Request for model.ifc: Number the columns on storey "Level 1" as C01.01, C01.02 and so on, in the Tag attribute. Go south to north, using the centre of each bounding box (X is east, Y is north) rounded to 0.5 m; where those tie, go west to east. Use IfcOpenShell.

First a look at what the model holds.

```python
import ifcopenshell
import ifcopenshell.util.element
import ifcopenshell.util.placement

model = ifcopenshell.open("model.ifc")
print(model.schema)
storey = next(s for s in model.by_type("IfcBuildingStorey") if s.Name == "Level 1")
columns = [e for e in ifcopenshell.util.element.get_decomposition(storey) if e.is_a("IfcColumn")]
for e in sorted(columns, key=lambda e: e.id()):
    origin = ifcopenshell.util.placement.get_local_placement(e.ObjectPlacement)[:3, 3]
    print(e.id(), e.Tag, e.Name, origin.round(2) + 0.0, sep=" | ")
```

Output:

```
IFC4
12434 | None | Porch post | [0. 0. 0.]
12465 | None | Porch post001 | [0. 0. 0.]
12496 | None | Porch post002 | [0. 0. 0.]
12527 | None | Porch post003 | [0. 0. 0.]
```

```python
import ifcopenshell
import ifcopenshell.geom
import ifcopenshell.util.element
import ifcopenshell.util.shape

model = ifcopenshell.open("model.ifc")
settings = ifcopenshell.geom.settings()
settings.set("use-world-coords", True)


def centre(element):
    shape = ifcopenshell.geom.create_shape(settings, element)
    return ifcopenshell.util.shape.get_bbox_centroid(shape.geometry)


storey = next(s for s in model.by_type("IfcBuildingStorey") if s.Name == "Level 1")
columns = [e for e in ifcopenshell.util.element.get_decomposition(storey) if e.is_a("IfcColumn")]

# Insertion points can sit at a corner or the storey origin, so sort by the geometry (in metres).
centres = {e: centre(e) for e in columns}
columns.sort(key=lambda e: (round(centres[e][1] / 0.5), centres[e][0]))

for i, e in enumerate(columns, start=1):
    number = f"C01.{i:02d}"
    e.Tag = number
    print(e.id(), number)

model.write("model_updated.ifc")
```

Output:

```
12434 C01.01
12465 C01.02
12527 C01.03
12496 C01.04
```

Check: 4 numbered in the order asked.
